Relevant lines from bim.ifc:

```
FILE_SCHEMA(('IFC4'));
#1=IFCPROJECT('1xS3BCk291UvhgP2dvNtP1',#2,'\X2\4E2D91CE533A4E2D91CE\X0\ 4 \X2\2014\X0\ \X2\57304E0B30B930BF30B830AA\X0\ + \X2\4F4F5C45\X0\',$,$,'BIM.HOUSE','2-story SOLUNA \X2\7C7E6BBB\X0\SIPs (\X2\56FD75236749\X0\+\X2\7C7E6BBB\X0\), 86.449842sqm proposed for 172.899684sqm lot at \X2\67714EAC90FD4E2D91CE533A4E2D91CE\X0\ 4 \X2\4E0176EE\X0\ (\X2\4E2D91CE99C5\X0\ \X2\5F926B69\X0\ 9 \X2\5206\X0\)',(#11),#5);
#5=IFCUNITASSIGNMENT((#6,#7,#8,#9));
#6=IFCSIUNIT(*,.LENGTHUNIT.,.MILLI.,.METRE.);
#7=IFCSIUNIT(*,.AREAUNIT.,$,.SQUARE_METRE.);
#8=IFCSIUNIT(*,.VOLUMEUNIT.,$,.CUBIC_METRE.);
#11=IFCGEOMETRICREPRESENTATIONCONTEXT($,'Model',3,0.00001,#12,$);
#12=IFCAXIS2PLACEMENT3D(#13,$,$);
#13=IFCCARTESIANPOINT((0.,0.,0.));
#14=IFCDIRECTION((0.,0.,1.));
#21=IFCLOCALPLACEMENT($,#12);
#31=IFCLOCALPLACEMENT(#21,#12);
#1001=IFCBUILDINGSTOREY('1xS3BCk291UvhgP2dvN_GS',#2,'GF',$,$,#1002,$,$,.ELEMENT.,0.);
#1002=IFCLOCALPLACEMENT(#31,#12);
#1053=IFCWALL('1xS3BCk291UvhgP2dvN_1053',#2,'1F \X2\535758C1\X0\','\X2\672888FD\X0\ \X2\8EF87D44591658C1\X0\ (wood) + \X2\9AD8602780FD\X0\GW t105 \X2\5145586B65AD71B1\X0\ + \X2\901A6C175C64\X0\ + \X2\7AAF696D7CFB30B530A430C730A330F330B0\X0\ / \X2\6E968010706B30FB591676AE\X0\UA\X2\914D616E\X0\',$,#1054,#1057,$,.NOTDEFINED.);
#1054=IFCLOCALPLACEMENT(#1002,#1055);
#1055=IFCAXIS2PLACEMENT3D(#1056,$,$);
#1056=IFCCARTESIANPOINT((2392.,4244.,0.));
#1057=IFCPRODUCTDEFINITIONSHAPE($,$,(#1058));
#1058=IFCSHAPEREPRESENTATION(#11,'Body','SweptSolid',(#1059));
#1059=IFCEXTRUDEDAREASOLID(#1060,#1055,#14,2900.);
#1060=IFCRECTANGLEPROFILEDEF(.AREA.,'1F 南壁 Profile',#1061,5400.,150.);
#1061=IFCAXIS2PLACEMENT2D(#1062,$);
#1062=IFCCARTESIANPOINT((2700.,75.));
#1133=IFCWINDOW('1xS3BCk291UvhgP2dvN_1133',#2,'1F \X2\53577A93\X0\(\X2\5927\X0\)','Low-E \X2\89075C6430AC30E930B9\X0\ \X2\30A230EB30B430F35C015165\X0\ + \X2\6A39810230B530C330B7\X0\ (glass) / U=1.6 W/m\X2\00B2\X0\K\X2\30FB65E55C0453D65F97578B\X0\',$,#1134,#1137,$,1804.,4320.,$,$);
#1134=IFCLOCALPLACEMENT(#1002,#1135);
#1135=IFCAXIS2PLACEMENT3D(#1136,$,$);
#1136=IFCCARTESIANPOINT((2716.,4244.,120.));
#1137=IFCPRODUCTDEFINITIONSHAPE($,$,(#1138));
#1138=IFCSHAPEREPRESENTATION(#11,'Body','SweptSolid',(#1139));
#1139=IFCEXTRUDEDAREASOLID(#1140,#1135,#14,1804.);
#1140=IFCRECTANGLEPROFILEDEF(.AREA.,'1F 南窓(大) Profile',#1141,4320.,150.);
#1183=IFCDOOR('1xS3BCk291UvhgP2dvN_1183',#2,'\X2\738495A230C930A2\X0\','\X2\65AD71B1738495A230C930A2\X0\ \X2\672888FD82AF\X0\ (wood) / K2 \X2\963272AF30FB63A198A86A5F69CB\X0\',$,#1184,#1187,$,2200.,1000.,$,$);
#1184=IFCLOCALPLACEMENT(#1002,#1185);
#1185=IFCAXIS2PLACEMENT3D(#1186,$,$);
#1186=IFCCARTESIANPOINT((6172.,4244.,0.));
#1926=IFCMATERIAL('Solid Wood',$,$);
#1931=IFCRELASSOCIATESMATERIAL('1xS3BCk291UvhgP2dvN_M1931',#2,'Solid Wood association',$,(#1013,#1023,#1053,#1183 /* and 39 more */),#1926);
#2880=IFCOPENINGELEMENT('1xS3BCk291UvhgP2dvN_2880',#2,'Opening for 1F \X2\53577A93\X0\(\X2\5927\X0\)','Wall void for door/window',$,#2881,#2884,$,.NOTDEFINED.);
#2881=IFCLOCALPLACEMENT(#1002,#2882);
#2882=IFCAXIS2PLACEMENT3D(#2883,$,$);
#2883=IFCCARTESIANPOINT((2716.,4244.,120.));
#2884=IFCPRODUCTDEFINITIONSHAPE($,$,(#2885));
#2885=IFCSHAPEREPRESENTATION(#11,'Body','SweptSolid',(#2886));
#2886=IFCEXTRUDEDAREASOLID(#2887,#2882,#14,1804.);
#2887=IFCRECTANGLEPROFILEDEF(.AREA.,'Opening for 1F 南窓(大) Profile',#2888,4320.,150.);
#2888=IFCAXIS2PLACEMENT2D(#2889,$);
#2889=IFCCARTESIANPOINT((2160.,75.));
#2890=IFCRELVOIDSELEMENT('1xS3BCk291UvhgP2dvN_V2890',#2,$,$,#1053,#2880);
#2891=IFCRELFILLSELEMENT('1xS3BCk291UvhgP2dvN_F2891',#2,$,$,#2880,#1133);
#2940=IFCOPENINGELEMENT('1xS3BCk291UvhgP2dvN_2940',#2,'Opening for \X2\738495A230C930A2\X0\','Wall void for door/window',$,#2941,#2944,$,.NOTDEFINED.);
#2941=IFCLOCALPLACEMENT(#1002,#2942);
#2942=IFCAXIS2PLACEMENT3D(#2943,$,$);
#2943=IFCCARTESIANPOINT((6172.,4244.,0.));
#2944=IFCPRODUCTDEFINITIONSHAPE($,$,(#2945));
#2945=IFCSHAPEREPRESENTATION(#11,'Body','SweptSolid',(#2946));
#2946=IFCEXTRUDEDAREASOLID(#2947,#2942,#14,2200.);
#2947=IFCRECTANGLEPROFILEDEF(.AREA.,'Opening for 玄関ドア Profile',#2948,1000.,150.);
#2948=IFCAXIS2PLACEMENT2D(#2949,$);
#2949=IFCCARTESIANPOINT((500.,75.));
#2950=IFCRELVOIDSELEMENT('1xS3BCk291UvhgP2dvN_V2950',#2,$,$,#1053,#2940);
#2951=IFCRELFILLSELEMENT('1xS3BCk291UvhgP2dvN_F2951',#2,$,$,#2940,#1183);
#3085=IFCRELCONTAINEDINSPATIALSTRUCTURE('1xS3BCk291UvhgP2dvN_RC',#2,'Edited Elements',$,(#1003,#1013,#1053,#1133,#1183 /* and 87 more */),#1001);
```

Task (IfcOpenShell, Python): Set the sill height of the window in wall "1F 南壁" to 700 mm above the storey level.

```python
import numpy as np
import ifcopenshell
import ifcopenshell.api.geometry
import ifcopenshell.geom
import ifcopenshell.util.element
import ifcopenshell.util.placement
import ifcopenshell.util.shape
import ifcopenshell.util.unit

model = ifcopenshell.open("bim.ifc")
unit_scale = ifcopenshell.util.unit.calculate_unit_scale(model)

window = model.by_guid("1xS3BCk291UvhgP2dvN_1133")
opening = window.FillsVoids[0].RelatingOpeningElement
storey = ifcopenshell.util.element.get_container(window, ifc_class="IfcBuildingStorey")
level = ifcopenshell.util.placement.get_local_placement(storey.ObjectPlacement)[2, 3]

# The opening's origin need not be at the sill, so measure its lowest point.
shape = ifcopenshell.geom.create_shape(ifcopenshell.geom.settings(), opening)
bottom = ifcopenshell.util.shape.get_shape_bottom_elevation(shape, shape.geometry) / unit_scale
dz = level + 700.0 - bottom

shift = np.array([0.0, 0.0, dz])
# The window is not placed relative to its opening, so move both.
for product in (opening, window):
    matrix = ifcopenshell.util.placement.get_local_placement(product.ObjectPlacement)
    matrix[:3, 3] += shift
    ifcopenshell.api.geometry.edit_object_placement(model, product=product, matrix=matrix, is_si=False)

print(f"moved by {dz * unit_scale:+.3f} m")

model.write("bim_edited.ifc")
```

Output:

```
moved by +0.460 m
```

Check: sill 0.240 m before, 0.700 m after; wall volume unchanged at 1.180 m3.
